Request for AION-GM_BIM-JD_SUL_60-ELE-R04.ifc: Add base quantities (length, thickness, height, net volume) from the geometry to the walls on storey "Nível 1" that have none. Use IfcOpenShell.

First a look at what the model holds.

```python
import ifcopenshell
import ifcopenshell.util.element
import ifcopenshell.util.unit

model = ifcopenshell.open("AION-GM_BIM-JD_SUL_60-ELE-R04.ifc")
print(model.schema)
for unit_type in ("LENGTHUNIT", "AREAUNIT", "VOLUMEUNIT"):
    print(unit_type, ifcopenshell.util.unit.calculate_unit_scale(model, unit_type))
storey = next(s for s in model.by_type("IfcBuildingStorey") if s.Name == "Nível 1")
walls = [e for e in ifcopenshell.util.element.get_decomposition(storey) if e.is_a("IfcWall")]
for e in sorted(walls, key=lambda e: e.id()):
    print(e.id(), e.is_a(), e.Name, list(ifcopenshell.util.element.get_psets(e, qtos_only=True)), sep=" | ")
```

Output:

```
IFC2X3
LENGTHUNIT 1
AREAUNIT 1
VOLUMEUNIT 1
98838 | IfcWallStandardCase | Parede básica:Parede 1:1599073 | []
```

```python
import ifcopenshell
import ifcopenshell.api.pset
import ifcopenshell.geom
import ifcopenshell.util.element
import ifcopenshell.util.shape
import ifcopenshell.util.unit

model = ifcopenshell.open("AION-GM_BIM-JD_SUL_60-ELE-R04.ifc")
unit_scale = ifcopenshell.util.unit.calculate_unit_scale(model)
volume_scale = ifcopenshell.util.unit.calculate_unit_scale(model, "VOLUMEUNIT")
settings = ifcopenshell.geom.settings()

storey = next(s for s in model.by_type("IfcBuildingStorey") if s.Name == "Nível 1")
walls = [e for e in ifcopenshell.util.element.get_decomposition(storey) if e.is_a("IfcWall")]

for e in sorted(walls, key=lambda e: e.id()):
    if ifcopenshell.util.element.get_psets(e, qtos_only=True, should_inherit=False):
        continue
    # Geometry comes back in metres, in the element's own axes.
    shape = ifcopenshell.geom.create_shape(settings, e)
    values = {
        "Length": ifcopenshell.util.shape.get_x(shape.geometry) / unit_scale,
        "Width": ifcopenshell.util.shape.get_y(shape.geometry) / unit_scale,
        "Height": ifcopenshell.util.shape.get_z(shape.geometry) / unit_scale,
        "NetVolume": ifcopenshell.util.shape.get_volume(shape.geometry) / volume_scale,
    }
    qto = ifcopenshell.api.pset.add_qto(model, product=e, name="BaseQuantities")
    ifcopenshell.api.pset.edit_qto(model, qto=qto, properties=values)
    print(e.id(), {k: round(v, 3) for k, v in values.items()})

model.write("AION-GM_BIM-JD_SUL_60-ELE-R04_rev.ifc")
```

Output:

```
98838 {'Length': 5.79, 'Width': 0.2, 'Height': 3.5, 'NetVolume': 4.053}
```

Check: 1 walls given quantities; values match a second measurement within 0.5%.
